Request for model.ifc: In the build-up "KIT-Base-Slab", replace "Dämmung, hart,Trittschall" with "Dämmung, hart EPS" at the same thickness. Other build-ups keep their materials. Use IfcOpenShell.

First a look at what the model holds.

```python
import ifcopenshell
import ifcopenshell.util.element

model = ifcopenshell.open("model.ifc")
print(model.schema)
for layer_set in model.by_type("IfcMaterialLayerSet"):
    if layer_set.LayerSetName == "KIT-Base-Slab":
        for layer in layer_set.MaterialLayers:
            print(layer.id(), layer.Material and layer.Material.Name, layer.LayerThickness, sep=" | ")
        print(len(ifcopenshell.util.element.get_elements_by_material(model, layer_set)), "elements and types use it")
print(sorted(m.Name for m in model.by_type("IfcMaterial") if m.Name)[:60])
```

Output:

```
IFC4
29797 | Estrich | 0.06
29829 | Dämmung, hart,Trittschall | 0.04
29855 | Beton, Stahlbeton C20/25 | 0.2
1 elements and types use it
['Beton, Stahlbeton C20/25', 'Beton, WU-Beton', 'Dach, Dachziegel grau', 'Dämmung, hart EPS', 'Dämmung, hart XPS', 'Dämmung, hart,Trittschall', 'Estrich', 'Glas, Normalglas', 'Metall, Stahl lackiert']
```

```python
import ifcopenshell
import ifcopenshell.api.material

model = ifcopenshell.open("model.ifc")

layer_set = next(s for s in model.by_type("IfcMaterialLayerSet") if s.LayerSetName == "KIT-Base-Slab")
layer = next(l for l in layer_set.MaterialLayers if l.Material and l.Material.Name == "Dämmung, hart,Trittschall")
material = next(m for m in model.by_type("IfcMaterial") if m.Name == "Dämmung, hart EPS")

# Point this one layer at the other material; renaming the old one would change it everywhere.
ifcopenshell.api.material.edit_layer(model, layer=layer, attributes={}, material=material)

print([l.Material.Name if l.Material else None for l in layer_set.MaterialLayers])

model.write("model_updated.ifc")
```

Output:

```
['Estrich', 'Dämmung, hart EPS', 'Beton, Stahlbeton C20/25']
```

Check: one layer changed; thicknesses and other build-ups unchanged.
